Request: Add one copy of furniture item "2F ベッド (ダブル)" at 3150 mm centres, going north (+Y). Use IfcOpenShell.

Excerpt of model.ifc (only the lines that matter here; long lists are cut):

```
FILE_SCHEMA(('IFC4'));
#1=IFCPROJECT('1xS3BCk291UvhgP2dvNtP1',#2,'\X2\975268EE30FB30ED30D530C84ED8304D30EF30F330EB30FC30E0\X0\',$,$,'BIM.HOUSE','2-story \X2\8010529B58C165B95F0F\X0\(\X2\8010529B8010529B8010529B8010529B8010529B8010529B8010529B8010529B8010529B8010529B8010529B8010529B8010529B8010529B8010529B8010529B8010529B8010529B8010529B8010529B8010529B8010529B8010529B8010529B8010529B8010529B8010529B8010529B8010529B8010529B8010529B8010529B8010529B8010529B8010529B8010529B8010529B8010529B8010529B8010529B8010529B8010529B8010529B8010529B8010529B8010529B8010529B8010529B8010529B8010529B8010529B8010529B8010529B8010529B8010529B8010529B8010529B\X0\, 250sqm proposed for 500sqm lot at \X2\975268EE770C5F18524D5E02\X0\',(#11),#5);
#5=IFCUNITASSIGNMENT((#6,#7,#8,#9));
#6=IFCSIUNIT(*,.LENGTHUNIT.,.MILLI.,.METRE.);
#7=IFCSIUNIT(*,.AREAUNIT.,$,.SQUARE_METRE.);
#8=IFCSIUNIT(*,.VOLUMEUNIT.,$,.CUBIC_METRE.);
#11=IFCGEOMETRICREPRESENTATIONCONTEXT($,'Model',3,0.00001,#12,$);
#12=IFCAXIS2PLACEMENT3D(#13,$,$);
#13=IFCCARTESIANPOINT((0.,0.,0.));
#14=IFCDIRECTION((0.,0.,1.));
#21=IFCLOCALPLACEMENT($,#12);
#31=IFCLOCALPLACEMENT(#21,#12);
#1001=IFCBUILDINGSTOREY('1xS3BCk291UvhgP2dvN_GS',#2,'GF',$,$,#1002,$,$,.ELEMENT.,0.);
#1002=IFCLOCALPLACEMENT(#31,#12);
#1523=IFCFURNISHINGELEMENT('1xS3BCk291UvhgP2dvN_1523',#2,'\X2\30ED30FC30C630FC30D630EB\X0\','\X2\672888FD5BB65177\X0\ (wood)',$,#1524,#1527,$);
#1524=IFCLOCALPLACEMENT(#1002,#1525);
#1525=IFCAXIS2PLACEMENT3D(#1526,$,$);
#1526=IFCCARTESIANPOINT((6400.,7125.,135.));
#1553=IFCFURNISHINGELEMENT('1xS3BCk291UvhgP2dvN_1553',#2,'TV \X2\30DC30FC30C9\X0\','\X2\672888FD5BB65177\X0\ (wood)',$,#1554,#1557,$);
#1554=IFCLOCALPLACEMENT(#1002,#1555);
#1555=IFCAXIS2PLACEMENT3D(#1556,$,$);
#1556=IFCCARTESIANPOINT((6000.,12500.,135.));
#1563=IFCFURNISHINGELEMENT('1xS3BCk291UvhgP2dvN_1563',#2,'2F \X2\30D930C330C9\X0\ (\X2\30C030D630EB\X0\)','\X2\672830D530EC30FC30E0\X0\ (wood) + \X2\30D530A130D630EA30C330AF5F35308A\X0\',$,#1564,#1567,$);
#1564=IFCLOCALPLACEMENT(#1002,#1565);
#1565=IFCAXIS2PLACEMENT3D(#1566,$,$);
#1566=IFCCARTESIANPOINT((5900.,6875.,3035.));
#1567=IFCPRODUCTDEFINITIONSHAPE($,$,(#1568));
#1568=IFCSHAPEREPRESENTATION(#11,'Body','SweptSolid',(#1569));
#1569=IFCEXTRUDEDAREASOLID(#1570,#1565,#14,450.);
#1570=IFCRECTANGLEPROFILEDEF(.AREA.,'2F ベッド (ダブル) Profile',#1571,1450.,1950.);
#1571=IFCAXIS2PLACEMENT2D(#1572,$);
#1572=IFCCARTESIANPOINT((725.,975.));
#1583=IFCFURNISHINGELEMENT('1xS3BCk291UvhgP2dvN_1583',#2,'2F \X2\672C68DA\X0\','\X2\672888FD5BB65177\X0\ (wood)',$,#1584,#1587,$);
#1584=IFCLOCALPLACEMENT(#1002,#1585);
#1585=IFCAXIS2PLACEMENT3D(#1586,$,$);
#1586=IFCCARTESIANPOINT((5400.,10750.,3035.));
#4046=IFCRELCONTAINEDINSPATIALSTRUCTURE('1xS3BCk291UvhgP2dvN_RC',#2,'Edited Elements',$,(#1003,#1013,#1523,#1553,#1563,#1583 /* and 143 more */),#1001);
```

```python
import numpy as np
import ifcopenshell
import ifcopenshell.api.geometry
import ifcopenshell.api.root
import ifcopenshell.util.element
import ifcopenshell.util.placement
import ifcopenshell.util.unit

model = ifcopenshell.open("model.ifc")
unit_scale = ifcopenshell.util.unit.calculate_unit_scale(model)


def reuse_history(source, copy):
    """copy_class also copies each property set's owner history, people and application; keep the originals."""
    for rel in copy.IsDefinedBy:
        if rel.is_a("IfcRelDefinesByProperties") and (history := rel.RelatingPropertyDefinition.OwnerHistory):
            rel.RelatingPropertyDefinition.OwnerHistory = source.OwnerHistory
            ifcopenshell.util.element.remove_deep2(model, history)


source = model.by_guid("1xS3BCk291UvhgP2dvN_1563")
base = ifcopenshell.util.placement.get_local_placement(source.ObjectPlacement)
step = np.array([0.0, 1.0, 0.0]) * 3.15 / unit_scale

for i in range(1, 2):
    copy = ifcopenshell.api.root.copy_class(model, product=source)
    copy.Representation = ifcopenshell.util.element.copy_deep(
        model, source.Representation, exclude=["IfcGeometricRepresentationContext", "IfcRepresentationMap"]
    )
    reuse_history(source, copy)
    matrix = base.copy()
    matrix[:3, 3] += i * step
    print("added at", matrix[:3, 3].round(3) + 0.0)
    ifcopenshell.api.geometry.edit_object_placement(model, product=copy, matrix=matrix, is_si=False)

model.write("model_v2.ifc")
```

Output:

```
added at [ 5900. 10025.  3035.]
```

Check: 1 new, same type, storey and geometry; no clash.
